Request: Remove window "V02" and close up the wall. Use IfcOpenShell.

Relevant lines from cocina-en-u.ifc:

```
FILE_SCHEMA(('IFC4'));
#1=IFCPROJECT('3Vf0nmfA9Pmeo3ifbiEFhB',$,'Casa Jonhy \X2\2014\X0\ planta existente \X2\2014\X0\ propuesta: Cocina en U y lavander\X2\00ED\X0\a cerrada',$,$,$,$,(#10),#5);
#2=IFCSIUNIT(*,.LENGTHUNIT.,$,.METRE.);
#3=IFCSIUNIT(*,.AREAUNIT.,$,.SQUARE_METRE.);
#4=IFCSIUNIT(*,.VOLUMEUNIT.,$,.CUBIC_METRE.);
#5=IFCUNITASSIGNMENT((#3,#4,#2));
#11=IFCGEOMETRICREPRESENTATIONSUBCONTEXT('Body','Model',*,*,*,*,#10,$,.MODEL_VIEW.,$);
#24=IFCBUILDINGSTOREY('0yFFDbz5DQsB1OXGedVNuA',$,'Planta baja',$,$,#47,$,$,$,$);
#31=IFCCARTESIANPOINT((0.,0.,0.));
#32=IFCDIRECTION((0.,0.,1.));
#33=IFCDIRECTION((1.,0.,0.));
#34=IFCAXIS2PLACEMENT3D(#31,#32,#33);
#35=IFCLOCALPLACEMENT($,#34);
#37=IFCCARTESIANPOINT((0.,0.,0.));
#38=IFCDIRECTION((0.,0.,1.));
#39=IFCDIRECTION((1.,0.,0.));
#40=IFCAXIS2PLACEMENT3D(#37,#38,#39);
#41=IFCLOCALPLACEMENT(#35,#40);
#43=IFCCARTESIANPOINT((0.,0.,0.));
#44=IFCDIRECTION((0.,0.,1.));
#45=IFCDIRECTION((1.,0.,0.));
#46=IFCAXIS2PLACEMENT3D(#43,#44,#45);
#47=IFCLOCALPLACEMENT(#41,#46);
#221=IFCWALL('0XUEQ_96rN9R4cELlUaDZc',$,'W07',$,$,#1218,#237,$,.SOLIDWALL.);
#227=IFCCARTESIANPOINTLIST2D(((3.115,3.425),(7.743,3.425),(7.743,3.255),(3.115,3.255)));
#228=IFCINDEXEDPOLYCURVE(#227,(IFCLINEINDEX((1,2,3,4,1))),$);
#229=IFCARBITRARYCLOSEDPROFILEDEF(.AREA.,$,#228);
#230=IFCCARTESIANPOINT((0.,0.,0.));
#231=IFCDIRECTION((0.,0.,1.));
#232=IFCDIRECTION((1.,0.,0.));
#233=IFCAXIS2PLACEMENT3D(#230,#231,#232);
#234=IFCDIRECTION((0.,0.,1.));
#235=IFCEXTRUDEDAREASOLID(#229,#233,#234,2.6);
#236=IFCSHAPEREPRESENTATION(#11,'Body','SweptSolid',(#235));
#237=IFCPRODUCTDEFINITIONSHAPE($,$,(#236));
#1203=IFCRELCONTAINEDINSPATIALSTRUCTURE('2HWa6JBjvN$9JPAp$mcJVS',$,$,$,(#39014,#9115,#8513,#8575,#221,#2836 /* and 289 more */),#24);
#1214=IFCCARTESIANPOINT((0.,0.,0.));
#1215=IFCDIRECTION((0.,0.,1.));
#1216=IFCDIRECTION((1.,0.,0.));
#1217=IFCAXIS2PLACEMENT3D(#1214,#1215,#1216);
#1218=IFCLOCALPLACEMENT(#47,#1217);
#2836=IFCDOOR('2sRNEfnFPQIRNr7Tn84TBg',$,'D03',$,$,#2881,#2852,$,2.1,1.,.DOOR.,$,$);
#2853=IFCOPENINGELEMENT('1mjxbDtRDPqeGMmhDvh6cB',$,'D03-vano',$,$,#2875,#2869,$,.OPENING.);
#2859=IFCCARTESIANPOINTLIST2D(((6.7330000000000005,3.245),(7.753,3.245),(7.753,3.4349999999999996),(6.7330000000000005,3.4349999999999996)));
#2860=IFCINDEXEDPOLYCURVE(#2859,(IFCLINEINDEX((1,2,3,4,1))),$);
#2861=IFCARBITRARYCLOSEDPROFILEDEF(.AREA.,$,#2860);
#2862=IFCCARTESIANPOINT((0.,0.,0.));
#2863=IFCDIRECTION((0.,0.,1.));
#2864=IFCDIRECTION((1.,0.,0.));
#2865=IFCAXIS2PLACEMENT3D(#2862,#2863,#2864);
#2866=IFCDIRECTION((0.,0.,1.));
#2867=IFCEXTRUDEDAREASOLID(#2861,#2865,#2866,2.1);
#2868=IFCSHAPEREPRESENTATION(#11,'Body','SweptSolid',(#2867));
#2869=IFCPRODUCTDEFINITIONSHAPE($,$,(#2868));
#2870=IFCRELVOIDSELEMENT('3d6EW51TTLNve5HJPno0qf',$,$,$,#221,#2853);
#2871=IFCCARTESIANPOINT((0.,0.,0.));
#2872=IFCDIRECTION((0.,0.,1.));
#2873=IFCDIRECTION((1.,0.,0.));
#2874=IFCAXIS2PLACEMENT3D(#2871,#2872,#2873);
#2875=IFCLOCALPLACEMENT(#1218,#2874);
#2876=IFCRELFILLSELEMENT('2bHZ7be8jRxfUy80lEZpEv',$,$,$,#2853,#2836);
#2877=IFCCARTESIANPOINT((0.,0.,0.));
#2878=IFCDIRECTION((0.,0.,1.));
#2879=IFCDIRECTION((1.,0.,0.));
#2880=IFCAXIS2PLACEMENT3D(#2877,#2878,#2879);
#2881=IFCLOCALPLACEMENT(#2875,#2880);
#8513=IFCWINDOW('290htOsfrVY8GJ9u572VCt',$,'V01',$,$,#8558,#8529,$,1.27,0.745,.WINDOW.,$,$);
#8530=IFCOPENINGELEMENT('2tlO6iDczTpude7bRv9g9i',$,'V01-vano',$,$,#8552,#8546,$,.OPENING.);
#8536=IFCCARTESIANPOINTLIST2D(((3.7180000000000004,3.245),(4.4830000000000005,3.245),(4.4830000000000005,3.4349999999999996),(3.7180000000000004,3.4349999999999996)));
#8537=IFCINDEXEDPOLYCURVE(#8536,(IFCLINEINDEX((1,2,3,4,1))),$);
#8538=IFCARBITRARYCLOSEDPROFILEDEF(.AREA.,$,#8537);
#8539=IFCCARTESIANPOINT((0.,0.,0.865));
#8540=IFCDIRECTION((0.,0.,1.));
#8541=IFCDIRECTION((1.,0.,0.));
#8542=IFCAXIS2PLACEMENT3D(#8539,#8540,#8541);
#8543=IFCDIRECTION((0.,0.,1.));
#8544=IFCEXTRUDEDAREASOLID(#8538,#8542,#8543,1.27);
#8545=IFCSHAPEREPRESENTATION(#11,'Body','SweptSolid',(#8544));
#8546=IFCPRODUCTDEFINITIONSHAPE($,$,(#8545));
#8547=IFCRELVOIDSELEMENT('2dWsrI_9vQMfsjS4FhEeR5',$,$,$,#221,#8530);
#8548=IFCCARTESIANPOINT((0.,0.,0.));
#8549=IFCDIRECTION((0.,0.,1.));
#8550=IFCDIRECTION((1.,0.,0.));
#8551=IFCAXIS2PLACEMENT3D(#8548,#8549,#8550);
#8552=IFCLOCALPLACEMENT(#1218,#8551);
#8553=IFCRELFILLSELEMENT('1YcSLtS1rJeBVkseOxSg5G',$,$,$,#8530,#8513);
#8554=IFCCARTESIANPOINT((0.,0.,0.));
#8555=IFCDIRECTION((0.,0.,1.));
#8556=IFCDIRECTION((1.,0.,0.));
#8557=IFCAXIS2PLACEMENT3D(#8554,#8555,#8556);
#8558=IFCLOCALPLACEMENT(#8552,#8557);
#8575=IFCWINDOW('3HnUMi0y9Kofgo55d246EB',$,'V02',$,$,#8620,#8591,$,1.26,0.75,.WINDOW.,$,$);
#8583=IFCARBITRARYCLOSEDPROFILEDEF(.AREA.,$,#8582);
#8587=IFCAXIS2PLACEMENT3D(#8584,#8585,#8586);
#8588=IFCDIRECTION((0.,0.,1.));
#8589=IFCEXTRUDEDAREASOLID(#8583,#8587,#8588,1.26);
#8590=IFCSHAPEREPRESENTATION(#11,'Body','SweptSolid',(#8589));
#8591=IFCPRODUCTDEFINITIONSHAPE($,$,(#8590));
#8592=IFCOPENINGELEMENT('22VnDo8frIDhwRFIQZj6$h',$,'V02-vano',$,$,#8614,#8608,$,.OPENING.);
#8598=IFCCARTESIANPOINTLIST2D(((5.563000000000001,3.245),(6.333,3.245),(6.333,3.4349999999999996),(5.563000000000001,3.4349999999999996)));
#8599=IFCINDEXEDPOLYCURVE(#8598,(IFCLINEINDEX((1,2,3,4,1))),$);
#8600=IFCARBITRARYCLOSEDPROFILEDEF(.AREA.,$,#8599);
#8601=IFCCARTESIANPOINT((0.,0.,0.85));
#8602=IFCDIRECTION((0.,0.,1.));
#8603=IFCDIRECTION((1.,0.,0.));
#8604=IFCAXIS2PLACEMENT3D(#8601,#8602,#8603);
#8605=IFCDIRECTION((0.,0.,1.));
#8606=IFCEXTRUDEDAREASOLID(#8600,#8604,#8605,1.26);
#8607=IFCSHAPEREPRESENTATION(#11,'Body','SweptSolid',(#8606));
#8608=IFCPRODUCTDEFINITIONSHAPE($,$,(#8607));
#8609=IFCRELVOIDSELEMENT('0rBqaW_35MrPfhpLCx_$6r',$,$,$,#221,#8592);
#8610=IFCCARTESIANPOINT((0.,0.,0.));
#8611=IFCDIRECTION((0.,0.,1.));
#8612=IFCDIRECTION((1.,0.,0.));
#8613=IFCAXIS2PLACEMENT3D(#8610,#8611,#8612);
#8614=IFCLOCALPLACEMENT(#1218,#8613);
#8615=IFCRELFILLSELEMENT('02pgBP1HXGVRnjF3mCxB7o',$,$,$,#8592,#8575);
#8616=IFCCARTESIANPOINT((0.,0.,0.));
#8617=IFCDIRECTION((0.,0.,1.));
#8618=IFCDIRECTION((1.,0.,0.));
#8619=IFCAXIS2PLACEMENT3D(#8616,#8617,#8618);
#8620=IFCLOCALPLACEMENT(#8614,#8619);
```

```python
import ifcopenshell
import ifcopenshell.api.feature
import ifcopenshell.api.root
import ifcopenshell.geom
import ifcopenshell.util.shape

model = ifcopenshell.open("cocina-en-u.ifc")
settings = ifcopenshell.geom.settings()


def volume(element):
    """Net volume in cubic metres, openings subtracted."""
    shape = ifcopenshell.geom.create_shape(settings, element)
    return ifcopenshell.util.shape.get_volume(shape.geometry)


window = model.by_guid("3HnUMi0y9Kofgo55d246EB")
opening = window.FillsVoids[0].RelatingOpeningElement
wall = opening.VoidsElements[0].RelatingBuildingElement
before = volume(wall)

ifcopenshell.api.root.remove_product(model, product=window)
ifcopenshell.api.feature.remove_feature(model, feature=opening)

after = volume(wall)

print(f"wall volume {before:.3f} -> {after:.3f} m3")

model.write("cocina-en-u_edited.ifc")
```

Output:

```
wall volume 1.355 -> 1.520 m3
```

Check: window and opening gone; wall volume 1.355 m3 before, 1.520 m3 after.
